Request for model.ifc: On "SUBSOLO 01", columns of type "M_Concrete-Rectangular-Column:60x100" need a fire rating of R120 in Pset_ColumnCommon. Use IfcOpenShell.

First a look at what the model holds.

```python
import ifcopenshell
import ifcopenshell.util.element

model = ifcopenshell.open("model.ifc")
print(model.schema)
storey = next(s for s in model.by_type("IfcBuildingStorey") if s.Name == "SUBSOLO 01")
columns = [e for e in ifcopenshell.util.element.get_decomposition(storey) if e.is_a("IfcColumn")]
seen = {}
for e in columns:
    element_type = ifcopenshell.util.element.get_type(e)
    key = (element_type.Name if element_type != e and element_type else None, ifcopenshell.util.element.get_pset(e, "Pset_ColumnCommon", "FireRating"))
    seen[key] = seen.get(key, 0) + 1
for (name, value), count in sorted(seen.items(), key=str):
    print(count, "x", name, "|", value)
```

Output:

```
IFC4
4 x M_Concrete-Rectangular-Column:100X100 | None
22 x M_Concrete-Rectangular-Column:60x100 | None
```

```python
import ifcopenshell
import ifcopenshell.api.pset
import ifcopenshell.util.element

model = ifcopenshell.open("model.ifc")

storey = next(s for s in model.by_type("IfcBuildingStorey") if s.Name == "SUBSOLO 01")
columns = [e for e in ifcopenshell.util.element.get_decomposition(storey) if e.is_a("IfcColumn")]

count = 0
for e in columns:
    element_type = ifcopenshell.util.element.get_type(e)
    if element_type in (None, e) or element_type.Name != "M_Concrete-Rectangular-Column:60x100":
        continue
    # add_pset returns the element's existing set when there is one.
    pset = ifcopenshell.api.pset.add_pset(model, product=e, name="Pset_ColumnCommon")
    ifcopenshell.api.pset.edit_pset(model, pset=pset, properties={"FireRating": "R120"})
    count += 1

print(count, "columns updated")

model.write("model_rev.ifc")
```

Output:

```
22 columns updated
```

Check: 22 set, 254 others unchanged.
